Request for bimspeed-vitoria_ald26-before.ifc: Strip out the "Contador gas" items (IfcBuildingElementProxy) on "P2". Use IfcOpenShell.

First a look at what the model holds.

```python
import ifcopenshell
import ifcopenshell.util.element

model = ifcopenshell.open("bimspeed-vitoria_ald26-before.ifc")
print(model.schema)
storey = next(s for s in model.by_type("IfcBuildingStorey") if s.Name == "P2")
proxies = [e for e in ifcopenshell.util.element.get_decomposition(storey) if e.is_a("IfcBuildingElementProxy")]
seen = {}
for e in proxies:
    element_type = ifcopenshell.util.element.get_type(e)
    name = element_type.Name if element_type not in (None, e) else None
    seen[name] = seen.get(name, 0) + 1
for name, count in sorted(seen.items(), key=str):
    print(count, "x", name)
```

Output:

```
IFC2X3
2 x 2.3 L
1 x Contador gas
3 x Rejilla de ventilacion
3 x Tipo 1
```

```python
import ifcopenshell
import ifcopenshell.api.root
import ifcopenshell.util.element

model = ifcopenshell.open("bimspeed-vitoria_ald26-before.ifc")

storey = next(s for s in model.by_type("IfcBuildingStorey") if s.Name == "P2")
proxies = [e for e in ifcopenshell.util.element.get_decomposition(storey) if e.is_a("IfcBuildingElementProxy")]
targets = [e for e in proxies if (t := ifcopenshell.util.element.get_type(e)) not in (None, e) and t.Name == "Contador gas"]

for e in targets:
    ifcopenshell.api.root.remove_product(model, product=e)
print(len(targets), "removed")

model.write("bimspeed-vitoria_ald26-before_edited.ifc")
```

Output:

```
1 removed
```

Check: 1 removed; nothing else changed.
